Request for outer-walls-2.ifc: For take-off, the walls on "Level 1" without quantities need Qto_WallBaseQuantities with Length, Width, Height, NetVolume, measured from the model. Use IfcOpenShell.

First a look at what the model holds.

```python
import ifcopenshell
import ifcopenshell.util.element
import ifcopenshell.util.unit

model = ifcopenshell.open("outer-walls-2.ifc")
print(model.schema)
for unit_type in ("LENGTHUNIT", "AREAUNIT", "VOLUMEUNIT"):
    print(unit_type, ifcopenshell.util.unit.calculate_unit_scale(model, unit_type))
storey = next(s for s in model.by_type("IfcBuildingStorey") if s.Name == "Level 1")
walls = [e for e in ifcopenshell.util.element.get_decomposition(storey) if e.is_a("IfcWall")]
for e in sorted(walls, key=lambda e: e.id()):
    print(e.id(), e.is_a(), e.Name, list(ifcopenshell.util.element.get_psets(e, qtos_only=True)), sep=" | ")
```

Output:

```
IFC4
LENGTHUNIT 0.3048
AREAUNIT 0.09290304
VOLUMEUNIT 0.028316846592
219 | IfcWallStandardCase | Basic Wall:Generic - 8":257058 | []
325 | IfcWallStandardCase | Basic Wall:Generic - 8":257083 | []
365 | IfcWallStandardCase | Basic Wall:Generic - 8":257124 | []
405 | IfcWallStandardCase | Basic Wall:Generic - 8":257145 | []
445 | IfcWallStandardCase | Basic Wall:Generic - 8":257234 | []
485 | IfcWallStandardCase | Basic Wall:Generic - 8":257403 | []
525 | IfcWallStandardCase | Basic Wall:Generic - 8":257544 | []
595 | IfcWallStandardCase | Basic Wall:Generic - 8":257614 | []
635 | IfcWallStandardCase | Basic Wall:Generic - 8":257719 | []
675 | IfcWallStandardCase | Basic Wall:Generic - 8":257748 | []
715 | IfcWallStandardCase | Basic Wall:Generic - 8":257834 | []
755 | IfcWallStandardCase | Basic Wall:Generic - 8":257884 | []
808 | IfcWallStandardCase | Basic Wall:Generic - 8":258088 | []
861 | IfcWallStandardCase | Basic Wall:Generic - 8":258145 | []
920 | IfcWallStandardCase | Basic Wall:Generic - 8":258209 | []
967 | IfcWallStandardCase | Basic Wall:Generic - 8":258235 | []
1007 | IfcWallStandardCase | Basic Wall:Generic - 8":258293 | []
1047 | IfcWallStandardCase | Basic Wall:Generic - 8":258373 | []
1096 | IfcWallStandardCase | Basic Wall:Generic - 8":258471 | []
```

```python
import ifcopenshell
import ifcopenshell.api.pset
import ifcopenshell.geom
import ifcopenshell.util.element
import ifcopenshell.util.shape
import ifcopenshell.util.unit

model = ifcopenshell.open("outer-walls-2.ifc")
unit_scale = ifcopenshell.util.unit.calculate_unit_scale(model)
volume_scale = ifcopenshell.util.unit.calculate_unit_scale(model, "VOLUMEUNIT")
settings = ifcopenshell.geom.settings()

storey = next(s for s in model.by_type("IfcBuildingStorey") if s.Name == "Level 1")
walls = [e for e in ifcopenshell.util.element.get_decomposition(storey) if e.is_a("IfcWall")]

for e in sorted(walls, key=lambda e: e.id()):
    if ifcopenshell.util.element.get_psets(e, qtos_only=True, should_inherit=False):
        continue
    # Geometry comes back in metres, in the element's own axes.
    shape = ifcopenshell.geom.create_shape(settings, e)
    values = {
        "Length": ifcopenshell.util.shape.get_x(shape.geometry) / unit_scale,
        "Width": ifcopenshell.util.shape.get_y(shape.geometry) / unit_scale,
        "Height": ifcopenshell.util.shape.get_z(shape.geometry) / unit_scale,
        "NetVolume": ifcopenshell.util.shape.get_volume(shape.geometry) / volume_scale,
    }
    qto = ifcopenshell.api.pset.add_qto(model, product=e, name="Qto_WallBaseQuantities")
    ifcopenshell.api.pset.edit_qto(model, qto=qto, properties=values)
    print(e.id(), {k: round(v, 3) for k, v in values.items()})

model.write("outer-walls-2_updated.ifc")
```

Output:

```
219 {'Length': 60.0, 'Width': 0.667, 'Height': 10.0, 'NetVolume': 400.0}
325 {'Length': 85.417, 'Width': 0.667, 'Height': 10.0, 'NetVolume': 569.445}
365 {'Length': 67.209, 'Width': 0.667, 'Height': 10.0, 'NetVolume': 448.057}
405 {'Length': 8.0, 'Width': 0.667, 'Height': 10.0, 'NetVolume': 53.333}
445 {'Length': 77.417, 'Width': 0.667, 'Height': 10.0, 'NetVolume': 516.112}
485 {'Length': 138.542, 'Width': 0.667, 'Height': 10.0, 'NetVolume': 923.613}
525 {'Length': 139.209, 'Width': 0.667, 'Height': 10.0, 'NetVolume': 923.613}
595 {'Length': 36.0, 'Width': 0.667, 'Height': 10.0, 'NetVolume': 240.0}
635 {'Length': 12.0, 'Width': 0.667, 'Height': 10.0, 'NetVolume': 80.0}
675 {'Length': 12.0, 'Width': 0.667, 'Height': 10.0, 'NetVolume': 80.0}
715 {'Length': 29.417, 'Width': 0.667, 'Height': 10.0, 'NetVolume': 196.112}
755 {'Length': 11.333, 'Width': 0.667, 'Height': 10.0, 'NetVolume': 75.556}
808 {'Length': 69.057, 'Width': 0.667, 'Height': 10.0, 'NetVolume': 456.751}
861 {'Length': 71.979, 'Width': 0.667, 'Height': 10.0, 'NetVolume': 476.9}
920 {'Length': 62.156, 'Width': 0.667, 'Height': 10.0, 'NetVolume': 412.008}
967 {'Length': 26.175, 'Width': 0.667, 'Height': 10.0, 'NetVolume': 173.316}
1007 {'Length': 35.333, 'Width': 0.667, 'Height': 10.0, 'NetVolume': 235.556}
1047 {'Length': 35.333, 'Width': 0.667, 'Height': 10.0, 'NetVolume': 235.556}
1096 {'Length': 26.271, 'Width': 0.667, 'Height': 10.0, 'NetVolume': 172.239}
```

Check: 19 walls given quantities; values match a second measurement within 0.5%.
